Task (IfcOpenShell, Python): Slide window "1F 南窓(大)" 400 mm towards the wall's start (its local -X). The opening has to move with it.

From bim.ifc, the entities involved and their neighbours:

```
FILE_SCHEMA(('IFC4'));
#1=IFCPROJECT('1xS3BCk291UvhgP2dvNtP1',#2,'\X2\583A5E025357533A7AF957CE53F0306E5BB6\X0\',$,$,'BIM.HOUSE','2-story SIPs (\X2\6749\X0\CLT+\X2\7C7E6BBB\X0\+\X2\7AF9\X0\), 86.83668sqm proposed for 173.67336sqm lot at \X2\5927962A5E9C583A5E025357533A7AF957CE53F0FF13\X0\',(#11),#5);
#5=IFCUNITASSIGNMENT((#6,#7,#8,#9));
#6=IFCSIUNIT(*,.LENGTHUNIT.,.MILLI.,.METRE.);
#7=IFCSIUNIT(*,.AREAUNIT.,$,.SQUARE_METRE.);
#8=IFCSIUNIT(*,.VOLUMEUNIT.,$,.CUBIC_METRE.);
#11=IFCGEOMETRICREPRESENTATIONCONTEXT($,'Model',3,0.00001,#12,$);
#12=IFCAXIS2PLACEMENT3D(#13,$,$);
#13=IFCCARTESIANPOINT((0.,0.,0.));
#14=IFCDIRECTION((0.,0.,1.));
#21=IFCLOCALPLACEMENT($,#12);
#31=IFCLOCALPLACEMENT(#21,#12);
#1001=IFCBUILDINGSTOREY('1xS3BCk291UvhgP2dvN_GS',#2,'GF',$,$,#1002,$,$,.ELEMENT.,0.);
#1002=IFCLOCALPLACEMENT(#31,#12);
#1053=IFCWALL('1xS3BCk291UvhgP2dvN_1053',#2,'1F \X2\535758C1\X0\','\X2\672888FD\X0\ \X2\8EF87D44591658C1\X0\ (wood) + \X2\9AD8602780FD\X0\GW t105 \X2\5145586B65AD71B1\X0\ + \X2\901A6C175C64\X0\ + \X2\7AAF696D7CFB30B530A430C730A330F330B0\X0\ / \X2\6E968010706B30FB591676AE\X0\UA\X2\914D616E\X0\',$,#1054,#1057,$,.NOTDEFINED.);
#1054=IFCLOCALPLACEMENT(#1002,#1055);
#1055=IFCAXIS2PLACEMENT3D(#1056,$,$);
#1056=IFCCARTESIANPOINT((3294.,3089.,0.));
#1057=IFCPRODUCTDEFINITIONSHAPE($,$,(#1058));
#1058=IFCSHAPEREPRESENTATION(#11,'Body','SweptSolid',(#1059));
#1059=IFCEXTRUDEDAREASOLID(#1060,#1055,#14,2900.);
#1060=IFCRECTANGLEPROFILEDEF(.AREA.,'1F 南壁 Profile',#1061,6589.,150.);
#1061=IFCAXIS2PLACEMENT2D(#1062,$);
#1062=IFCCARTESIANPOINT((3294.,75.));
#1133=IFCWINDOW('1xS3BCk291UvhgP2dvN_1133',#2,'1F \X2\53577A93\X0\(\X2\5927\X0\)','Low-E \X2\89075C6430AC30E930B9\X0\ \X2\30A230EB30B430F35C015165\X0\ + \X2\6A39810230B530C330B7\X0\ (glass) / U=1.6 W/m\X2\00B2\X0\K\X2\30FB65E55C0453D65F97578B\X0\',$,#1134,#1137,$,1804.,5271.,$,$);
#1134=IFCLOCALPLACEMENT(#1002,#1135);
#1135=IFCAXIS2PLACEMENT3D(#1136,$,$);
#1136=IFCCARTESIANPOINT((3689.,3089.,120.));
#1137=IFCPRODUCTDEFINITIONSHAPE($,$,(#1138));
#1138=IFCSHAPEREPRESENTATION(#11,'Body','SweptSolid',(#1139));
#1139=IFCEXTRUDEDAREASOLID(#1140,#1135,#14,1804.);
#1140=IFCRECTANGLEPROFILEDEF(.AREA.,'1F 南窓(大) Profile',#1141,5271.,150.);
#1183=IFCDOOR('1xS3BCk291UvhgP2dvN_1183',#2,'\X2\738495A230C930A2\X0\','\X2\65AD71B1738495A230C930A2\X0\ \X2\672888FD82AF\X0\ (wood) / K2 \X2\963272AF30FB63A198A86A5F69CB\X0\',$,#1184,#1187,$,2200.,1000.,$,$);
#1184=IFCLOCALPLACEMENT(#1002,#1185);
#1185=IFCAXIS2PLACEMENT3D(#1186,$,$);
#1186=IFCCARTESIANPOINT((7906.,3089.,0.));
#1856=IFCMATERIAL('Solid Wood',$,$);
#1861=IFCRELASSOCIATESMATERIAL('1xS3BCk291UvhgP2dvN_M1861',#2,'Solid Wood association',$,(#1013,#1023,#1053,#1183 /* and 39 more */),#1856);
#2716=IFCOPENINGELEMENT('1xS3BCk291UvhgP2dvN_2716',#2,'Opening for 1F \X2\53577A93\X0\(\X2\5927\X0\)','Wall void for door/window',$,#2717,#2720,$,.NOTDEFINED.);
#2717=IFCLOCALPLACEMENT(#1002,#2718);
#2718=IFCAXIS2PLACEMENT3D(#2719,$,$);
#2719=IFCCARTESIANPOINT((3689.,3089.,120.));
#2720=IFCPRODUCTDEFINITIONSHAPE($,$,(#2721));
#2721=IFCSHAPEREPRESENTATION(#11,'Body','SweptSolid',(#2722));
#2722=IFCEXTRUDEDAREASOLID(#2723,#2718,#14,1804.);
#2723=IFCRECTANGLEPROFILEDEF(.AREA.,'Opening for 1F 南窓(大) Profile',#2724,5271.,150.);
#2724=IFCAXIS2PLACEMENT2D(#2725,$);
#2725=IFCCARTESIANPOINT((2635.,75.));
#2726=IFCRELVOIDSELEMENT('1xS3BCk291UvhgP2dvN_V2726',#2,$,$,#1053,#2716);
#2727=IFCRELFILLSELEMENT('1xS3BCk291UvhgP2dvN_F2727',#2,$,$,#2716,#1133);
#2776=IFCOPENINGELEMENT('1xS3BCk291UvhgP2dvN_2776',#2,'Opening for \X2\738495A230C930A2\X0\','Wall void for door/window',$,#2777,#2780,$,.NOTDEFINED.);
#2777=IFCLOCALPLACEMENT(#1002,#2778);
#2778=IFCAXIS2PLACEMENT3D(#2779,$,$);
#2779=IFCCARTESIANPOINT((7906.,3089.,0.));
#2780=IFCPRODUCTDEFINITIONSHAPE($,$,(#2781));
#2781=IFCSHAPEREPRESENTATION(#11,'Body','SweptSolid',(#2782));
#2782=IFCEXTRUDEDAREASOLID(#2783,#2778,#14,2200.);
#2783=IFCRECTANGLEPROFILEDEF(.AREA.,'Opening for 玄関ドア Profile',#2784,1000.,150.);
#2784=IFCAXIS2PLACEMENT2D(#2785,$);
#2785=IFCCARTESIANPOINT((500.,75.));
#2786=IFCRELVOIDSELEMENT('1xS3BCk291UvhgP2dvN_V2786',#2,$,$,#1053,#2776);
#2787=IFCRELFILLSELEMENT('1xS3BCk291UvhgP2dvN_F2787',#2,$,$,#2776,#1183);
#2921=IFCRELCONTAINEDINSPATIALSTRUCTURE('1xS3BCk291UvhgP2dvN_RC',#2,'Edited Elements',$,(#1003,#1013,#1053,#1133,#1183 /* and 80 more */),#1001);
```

```python
import ifcopenshell
import ifcopenshell.api.geometry
import ifcopenshell.util.placement
import ifcopenshell.util.unit

model = ifcopenshell.open("bim.ifc")
unit_scale = ifcopenshell.util.unit.calculate_unit_scale(model)

window = model.by_id(1133)
opening = window.FillsVoids[0].RelatingOpeningElement
wall = opening.VoidsElements[0].RelatingBuildingElement

wall_matrix = ifcopenshell.util.placement.get_local_placement(wall.ObjectPlacement)
shift = wall_matrix[:3, 0] * -0.4 / unit_scale
before = ifcopenshell.util.placement.get_local_placement(window.ObjectPlacement)[:3, 3].copy()

# The window is not placed relative to its opening, so move both.
for product in (opening, window):
    matrix = ifcopenshell.util.placement.get_local_placement(product.ObjectPlacement)
    matrix[:3, 3] += shift
    ifcopenshell.api.geometry.edit_object_placement(model, product=product, matrix=matrix, is_si=False)

after = ifcopenshell.util.placement.get_local_placement(window.ObjectPlacement)[:3, 3]
print("window moved by", (after - before).round(3) + 0.0)

model.write("bim_updated.ifc")
```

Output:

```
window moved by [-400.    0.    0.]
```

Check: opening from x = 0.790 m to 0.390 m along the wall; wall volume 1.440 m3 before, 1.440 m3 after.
